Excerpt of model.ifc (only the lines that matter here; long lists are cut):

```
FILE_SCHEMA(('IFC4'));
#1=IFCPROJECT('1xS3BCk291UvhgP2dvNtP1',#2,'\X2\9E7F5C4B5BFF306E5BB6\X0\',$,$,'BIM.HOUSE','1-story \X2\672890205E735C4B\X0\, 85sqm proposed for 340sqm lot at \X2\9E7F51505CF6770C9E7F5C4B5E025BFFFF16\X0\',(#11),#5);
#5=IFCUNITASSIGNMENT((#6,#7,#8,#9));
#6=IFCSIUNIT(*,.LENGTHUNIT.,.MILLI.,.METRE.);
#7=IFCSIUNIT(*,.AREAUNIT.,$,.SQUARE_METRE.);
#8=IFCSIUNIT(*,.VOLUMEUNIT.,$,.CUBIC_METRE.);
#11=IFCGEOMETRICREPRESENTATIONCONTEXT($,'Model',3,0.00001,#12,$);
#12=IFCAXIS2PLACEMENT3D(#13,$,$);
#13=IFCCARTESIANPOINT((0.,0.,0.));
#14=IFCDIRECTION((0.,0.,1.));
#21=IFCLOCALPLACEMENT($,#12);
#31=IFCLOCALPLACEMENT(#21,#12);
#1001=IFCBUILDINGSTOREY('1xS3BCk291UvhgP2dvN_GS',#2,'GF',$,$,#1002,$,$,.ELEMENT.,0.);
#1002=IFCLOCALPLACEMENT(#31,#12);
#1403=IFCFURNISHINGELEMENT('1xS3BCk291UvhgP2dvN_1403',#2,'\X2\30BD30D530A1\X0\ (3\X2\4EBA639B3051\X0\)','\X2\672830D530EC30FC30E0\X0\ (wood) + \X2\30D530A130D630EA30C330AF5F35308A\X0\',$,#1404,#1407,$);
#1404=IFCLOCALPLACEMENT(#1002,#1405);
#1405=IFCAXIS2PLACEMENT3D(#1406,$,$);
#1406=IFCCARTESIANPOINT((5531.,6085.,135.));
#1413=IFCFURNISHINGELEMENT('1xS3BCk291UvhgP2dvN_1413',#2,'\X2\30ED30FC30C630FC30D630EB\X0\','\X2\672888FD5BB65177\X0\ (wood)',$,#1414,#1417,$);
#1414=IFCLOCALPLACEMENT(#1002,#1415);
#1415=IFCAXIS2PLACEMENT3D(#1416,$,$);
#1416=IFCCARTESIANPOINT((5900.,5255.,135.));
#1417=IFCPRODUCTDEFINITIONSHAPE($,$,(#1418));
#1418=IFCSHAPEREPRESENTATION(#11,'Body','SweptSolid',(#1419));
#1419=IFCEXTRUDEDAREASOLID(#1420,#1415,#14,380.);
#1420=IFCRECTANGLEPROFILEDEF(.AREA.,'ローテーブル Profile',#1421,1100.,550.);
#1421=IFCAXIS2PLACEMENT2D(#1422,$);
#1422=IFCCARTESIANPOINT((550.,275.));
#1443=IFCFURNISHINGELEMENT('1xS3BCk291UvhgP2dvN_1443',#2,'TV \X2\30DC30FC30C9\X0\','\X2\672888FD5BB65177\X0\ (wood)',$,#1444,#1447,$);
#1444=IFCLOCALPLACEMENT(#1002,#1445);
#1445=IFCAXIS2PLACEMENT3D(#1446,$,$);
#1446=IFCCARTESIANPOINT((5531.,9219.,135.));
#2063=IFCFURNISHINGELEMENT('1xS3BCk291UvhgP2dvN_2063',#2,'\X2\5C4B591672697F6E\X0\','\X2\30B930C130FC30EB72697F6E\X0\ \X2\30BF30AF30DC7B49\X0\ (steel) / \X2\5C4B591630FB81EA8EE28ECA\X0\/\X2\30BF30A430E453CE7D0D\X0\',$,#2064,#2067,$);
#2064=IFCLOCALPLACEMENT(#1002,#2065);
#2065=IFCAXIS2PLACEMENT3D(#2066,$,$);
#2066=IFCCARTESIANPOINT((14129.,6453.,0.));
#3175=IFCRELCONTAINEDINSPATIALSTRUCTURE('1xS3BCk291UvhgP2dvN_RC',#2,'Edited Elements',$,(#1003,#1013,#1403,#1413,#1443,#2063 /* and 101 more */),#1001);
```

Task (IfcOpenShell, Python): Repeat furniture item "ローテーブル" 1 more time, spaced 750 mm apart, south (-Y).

```python
import numpy as np
import ifcopenshell
import ifcopenshell.api.geometry
import ifcopenshell.api.root
import ifcopenshell.util.element
import ifcopenshell.util.placement
import ifcopenshell.util.unit

model = ifcopenshell.open("model.ifc")
unit_scale = ifcopenshell.util.unit.calculate_unit_scale(model)


def reuse_history(source, copy):
    """copy_class also copies each property set's owner history, people and application; keep the originals."""
    for rel in copy.IsDefinedBy:
        if rel.is_a("IfcRelDefinesByProperties") and (history := rel.RelatingPropertyDefinition.OwnerHistory):
            rel.RelatingPropertyDefinition.OwnerHistory = source.OwnerHistory
            ifcopenshell.util.element.remove_deep2(model, history)


source = model.by_id(1413)
base = ifcopenshell.util.placement.get_local_placement(source.ObjectPlacement)
step = np.array([0.0, -1.0, 0.0]) * 0.75 / unit_scale

for i in range(1, 2):
    copy = ifcopenshell.api.root.copy_class(model, product=source)
    copy.Representation = ifcopenshell.util.element.copy_deep(
        model, source.Representation, exclude=["IfcGeometricRepresentationContext", "IfcRepresentationMap"]
    )
    reuse_history(source, copy)
    matrix = base.copy()
    matrix[:3, 3] += i * step
    print("added at", matrix[:3, 3].round(3) + 0.0)
    ifcopenshell.api.geometry.edit_object_placement(model, product=copy, matrix=matrix, is_si=False)

model.write("model_edited.ifc")
```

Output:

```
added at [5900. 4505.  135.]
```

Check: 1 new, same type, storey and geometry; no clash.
